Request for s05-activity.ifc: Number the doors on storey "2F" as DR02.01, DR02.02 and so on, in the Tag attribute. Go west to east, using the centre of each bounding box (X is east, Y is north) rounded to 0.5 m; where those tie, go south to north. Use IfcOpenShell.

First a look at what the model holds.

```python
import ifcopenshell
import ifcopenshell.util.element
import ifcopenshell.util.placement

model = ifcopenshell.open("s05-activity.ifc")
print(model.schema)
storey = next(s for s in model.by_type("IfcBuildingStorey") if s.Name == "2F")
doors = [e for e in ifcopenshell.util.element.get_decomposition(storey) if e.is_a("IfcDoor")]
for e in sorted(doors, key=lambda e: e.id()):
    origin = ifcopenshell.util.placement.get_local_placement(e.ObjectPlacement)[:3, 3]
    print(e.id(), e.Tag, e.Name, origin.round(2) + 0.0, sep=" | ")
```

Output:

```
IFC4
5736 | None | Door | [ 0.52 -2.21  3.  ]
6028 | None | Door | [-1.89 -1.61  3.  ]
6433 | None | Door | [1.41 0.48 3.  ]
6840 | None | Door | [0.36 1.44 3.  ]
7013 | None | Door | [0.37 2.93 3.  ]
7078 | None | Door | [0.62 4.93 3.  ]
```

```python
import ifcopenshell
import ifcopenshell.geom
import ifcopenshell.util.element
import ifcopenshell.util.shape

model = ifcopenshell.open("s05-activity.ifc")
settings = ifcopenshell.geom.settings()
settings.set("use-world-coords", True)


def centre(element):
    shape = ifcopenshell.geom.create_shape(settings, element)
    return ifcopenshell.util.shape.get_bbox_centroid(shape.geometry)


storey = next(s for s in model.by_type("IfcBuildingStorey") if s.Name == "2F")
doors = [e for e in ifcopenshell.util.element.get_decomposition(storey) if e.is_a("IfcDoor")]

# Insertion points can sit at a corner or the storey origin, so sort by the geometry (in metres).
centres = {e: centre(e) for e in doors}
doors.sort(key=lambda e: (round(centres[e][0] / 0.5), centres[e][1]))

for i, e in enumerate(doors, start=1):
    number = f"DR02.{i:02d}"
    e.Tag = number
    print(e.id(), number)

model.write("s05-activity-out.ifc")
```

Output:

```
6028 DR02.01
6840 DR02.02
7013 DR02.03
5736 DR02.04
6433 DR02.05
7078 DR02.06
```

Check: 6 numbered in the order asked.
